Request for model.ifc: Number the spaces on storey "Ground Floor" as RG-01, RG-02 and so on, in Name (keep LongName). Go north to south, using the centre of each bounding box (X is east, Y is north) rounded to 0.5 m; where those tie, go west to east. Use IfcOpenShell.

First a look at what the model holds.

```python
import ifcopenshell
import ifcopenshell.util.element
import ifcopenshell.util.placement

model = ifcopenshell.open("model.ifc")
print(model.schema)
storey = next(s for s in model.by_type("IfcBuildingStorey") if s.Name == "Ground Floor")
spaces = [e for e in ifcopenshell.util.element.get_decomposition(storey) if e.is_a("IfcSpace")]
for e in sorted(spaces, key=lambda e: e.id()):
    origin = ifcopenshell.util.placement.get_local_placement(e.ObjectPlacement)[:3, 3]
    print(e.id(), e.Name, e.LongName, origin.round(2) + 0.0, sep=" | ")
```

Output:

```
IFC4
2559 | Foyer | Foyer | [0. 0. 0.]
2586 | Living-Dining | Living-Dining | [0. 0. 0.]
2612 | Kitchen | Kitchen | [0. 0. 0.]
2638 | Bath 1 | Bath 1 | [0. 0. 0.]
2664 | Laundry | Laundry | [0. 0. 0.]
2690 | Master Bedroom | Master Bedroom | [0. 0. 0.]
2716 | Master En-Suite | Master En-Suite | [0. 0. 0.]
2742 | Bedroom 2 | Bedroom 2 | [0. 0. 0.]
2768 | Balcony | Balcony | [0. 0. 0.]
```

```python
import ifcopenshell
import ifcopenshell.geom
import ifcopenshell.util.element
import ifcopenshell.util.shape

model = ifcopenshell.open("model.ifc")
settings = ifcopenshell.geom.settings()
settings.set("use-world-coords", True)


def centre(element):
    shape = ifcopenshell.geom.create_shape(settings, element)
    return ifcopenshell.util.shape.get_bbox_centroid(shape.geometry)


storey = next(s for s in model.by_type("IfcBuildingStorey") if s.Name == "Ground Floor")
spaces = [e for e in ifcopenshell.util.element.get_decomposition(storey) if e.is_a("IfcSpace")]

# Insertion points can sit at a corner or the storey origin, so sort by the geometry (in metres).
centres = {e: centre(e) for e in spaces}
spaces.sort(key=lambda e: (-round(centres[e][1] / 0.5), centres[e][0]))

for i, e in enumerate(spaces, start=1):
    number = f"RG-{i:02d}"
    e.Name = number
    print(e.id(), number)

model.write("model_edited.ifc")
```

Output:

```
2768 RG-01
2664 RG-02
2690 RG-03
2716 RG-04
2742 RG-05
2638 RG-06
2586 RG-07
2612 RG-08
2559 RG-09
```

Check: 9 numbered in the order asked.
